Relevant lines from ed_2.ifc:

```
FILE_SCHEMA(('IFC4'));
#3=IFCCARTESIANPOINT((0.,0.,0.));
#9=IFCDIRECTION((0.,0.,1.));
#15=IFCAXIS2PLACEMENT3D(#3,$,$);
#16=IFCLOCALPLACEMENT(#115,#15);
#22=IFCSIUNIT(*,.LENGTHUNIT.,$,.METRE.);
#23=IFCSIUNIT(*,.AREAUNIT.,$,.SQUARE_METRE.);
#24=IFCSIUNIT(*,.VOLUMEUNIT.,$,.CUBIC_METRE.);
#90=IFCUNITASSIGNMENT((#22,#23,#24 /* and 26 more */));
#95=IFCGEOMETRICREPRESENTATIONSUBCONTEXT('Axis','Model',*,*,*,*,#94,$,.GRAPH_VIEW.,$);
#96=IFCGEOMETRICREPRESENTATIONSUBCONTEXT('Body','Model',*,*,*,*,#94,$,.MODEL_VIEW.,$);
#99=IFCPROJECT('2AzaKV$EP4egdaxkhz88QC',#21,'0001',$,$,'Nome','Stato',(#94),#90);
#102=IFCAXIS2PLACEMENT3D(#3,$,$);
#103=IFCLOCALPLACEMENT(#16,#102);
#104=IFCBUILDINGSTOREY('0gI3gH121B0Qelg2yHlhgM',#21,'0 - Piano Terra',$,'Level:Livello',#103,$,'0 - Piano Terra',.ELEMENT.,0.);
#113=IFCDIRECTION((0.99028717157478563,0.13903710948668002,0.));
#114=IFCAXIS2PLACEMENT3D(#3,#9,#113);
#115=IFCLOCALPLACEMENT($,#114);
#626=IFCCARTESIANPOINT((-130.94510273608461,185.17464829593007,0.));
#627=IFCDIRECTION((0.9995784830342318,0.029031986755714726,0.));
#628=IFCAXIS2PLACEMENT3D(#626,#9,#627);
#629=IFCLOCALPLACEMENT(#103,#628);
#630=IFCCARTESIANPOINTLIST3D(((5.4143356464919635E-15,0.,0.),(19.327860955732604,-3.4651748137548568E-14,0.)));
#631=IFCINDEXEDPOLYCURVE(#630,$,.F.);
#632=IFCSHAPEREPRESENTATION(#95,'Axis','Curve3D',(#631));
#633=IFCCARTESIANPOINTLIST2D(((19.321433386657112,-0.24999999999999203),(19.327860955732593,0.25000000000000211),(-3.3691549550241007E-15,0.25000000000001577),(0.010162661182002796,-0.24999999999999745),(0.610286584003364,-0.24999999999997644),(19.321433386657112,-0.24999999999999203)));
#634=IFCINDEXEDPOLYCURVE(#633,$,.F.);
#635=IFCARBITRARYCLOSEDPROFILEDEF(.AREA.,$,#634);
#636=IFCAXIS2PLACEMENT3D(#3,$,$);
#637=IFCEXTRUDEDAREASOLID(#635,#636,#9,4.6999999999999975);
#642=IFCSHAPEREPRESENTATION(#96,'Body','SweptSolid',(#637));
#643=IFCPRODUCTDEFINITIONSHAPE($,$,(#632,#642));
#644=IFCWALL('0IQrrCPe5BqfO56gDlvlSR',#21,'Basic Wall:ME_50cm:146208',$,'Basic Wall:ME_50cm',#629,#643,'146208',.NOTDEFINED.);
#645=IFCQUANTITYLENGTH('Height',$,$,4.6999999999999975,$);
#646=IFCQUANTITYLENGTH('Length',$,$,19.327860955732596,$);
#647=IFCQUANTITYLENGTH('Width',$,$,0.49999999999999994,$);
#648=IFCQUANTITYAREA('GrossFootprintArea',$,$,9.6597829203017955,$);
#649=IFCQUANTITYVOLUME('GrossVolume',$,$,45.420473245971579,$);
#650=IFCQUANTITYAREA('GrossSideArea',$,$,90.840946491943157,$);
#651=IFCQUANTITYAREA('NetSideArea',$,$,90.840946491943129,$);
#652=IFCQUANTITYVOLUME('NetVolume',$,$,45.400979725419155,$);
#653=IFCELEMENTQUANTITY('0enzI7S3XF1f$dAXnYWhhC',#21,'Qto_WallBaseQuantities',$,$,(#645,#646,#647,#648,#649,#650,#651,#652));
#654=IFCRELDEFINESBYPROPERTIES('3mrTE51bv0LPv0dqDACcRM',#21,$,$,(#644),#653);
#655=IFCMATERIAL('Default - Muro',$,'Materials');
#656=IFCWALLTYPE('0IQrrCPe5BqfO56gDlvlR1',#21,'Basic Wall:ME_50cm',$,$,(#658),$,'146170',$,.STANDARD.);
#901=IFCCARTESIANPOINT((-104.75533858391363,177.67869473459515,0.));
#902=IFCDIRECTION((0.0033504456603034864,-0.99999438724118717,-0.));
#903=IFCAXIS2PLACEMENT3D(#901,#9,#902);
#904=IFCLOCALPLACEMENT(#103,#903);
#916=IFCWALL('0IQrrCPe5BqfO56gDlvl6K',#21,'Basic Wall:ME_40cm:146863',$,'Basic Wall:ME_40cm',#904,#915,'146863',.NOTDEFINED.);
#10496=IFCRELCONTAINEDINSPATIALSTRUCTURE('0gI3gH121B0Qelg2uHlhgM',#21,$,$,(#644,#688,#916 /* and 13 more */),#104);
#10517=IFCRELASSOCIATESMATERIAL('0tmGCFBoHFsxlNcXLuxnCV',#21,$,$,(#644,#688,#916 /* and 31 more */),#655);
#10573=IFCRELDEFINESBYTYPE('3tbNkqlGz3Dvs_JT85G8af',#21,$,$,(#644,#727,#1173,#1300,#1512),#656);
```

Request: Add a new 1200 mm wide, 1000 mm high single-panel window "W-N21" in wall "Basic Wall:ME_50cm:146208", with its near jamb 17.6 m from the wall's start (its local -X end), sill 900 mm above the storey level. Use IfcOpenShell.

```python
import numpy as np
import ifcopenshell
import ifcopenshell.api.feature
import ifcopenshell.api.geometry
import ifcopenshell.api.pset
import ifcopenshell.api.root
import ifcopenshell.api.spatial
import ifcopenshell.geom
import ifcopenshell.util.element
import ifcopenshell.util.placement
import ifcopenshell.util.representation
import ifcopenshell.util.shape
import ifcopenshell.util.unit

model = ifcopenshell.open("ed_2.ifc")
unit_scale = ifcopenshell.util.unit.calculate_unit_scale(model)
area_scale = ifcopenshell.util.unit.calculate_unit_scale(model, "AREAUNIT")
volume_scale = ifcopenshell.util.unit.calculate_unit_scale(model, "VOLUMEUNIT")
settings = ifcopenshell.geom.settings()


def volume(element):
    """Net volume in cubic metres, openings subtracted."""
    shape = ifcopenshell.geom.create_shape(settings, element)
    return ifcopenshell.util.shape.get_volume(shape.geometry)


wall = model.by_guid("0IQrrCPe5BqfO56gDlvlSR")
storey = ifcopenshell.util.element.get_container(wall, ifc_class="IfcBuildingStorey")
context = ifcopenshell.util.representation.get_context(model, "Model", "Body", "MODEL_VIEW")
before = volume(wall)

width, height, from_end, sill = 1.2, 1, 17.6, 0.9  # metres

# The wall runs along its own X axis, and the end named is its -X end.
wall_shape = ifcopenshell.geom.create_shape(settings, wall)
x, y, z = ifcopenshell.util.shape.get_vertices(wall_shape.geometry).T
start = x.min() + from_end
face, thickness = float(y.min()), float(y.max() - y.min())
wall_matrix = ifcopenshell.util.placement.get_local_placement(wall.ObjectPlacement)
level = ifcopenshell.util.placement.get_local_placement(storey.ObjectPlacement)[2, 3]


def in_wall(x, y):
    """Placement at x, y metres in the wall's axes, at sill height."""
    matrix = wall_matrix.copy()
    matrix[:, 3] = wall_matrix @ np.array([x / unit_scale, y / unit_scale, 0.0, 1.0])
    matrix[2, 3] = level + sill / unit_scale
    return matrix


# Opening: a box that overshoots both wall faces by 50 mm.
opening = ifcopenshell.api.root.create_entity(model, ifc_class="IfcOpeningElement", predefined_type="OPENING")
box = ifcopenshell.api.geometry.add_wall_representation(
    model, context=context, length=width, height=height, thickness=thickness + 0.1
)
ifcopenshell.api.geometry.assign_representation(model, product=opening, representation=box)
ifcopenshell.api.geometry.edit_object_placement(model, product=opening, matrix=in_wall(start, face - 0.05), is_si=False)
ifcopenshell.api.feature.add_feature(model, feature=opening, element=wall)

window = ifcopenshell.api.root.create_entity(model, ifc_class="IfcWindow", name="W-N21", predefined_type="WINDOW")
window.OverallWidth, window.OverallHeight = width / unit_scale, height / unit_scale
window.PartitioningType = "SINGLE_PANEL"
body = ifcopenshell.api.geometry.add_window_representation(
    model,
    context=context,
    overall_width=window.OverallWidth,
    overall_height=window.OverallHeight,
    partition_type="SINGLE_PANEL",
)
ifcopenshell.api.geometry.assign_representation(model, product=window, representation=body)
ifcopenshell.api.spatial.assign_container(model, products=[window], relating_structure=storey)
ifcopenshell.api.feature.add_filling(model, opening=opening, element=window)

# Centre the window in the wall's thickness.
ifcopenshell.api.geometry.edit_object_placement(model, product=window, matrix=in_wall(start, face), is_si=False)
window_shape = ifcopenshell.geom.create_shape(settings, window)
depth = ifcopenshell.util.shape.get_vertices(window_shape.geometry)[:, 1]
offset = face + thickness / 2 - (depth.min() + depth.max()) / 2
ifcopenshell.api.geometry.edit_object_placement(model, product=window, matrix=in_wall(start, offset), is_si=False)

after = volume(wall)

# Update the wall's stored quantities.
qto = model.by_id(ifcopenshell.util.element.get_pset(wall, "Qto_WallBaseQuantities", should_inherit=False)["id"])
ifcopenshell.api.pset.edit_qto(model, qto=qto, properties={
    "NetSideArea": after / thickness / area_scale,
    "NetVolume": after / volume_scale,
})

print(f"wall volume {before:.3f} -> {after:.3f} m3")

model.write("ed_2_updated.ifc")
```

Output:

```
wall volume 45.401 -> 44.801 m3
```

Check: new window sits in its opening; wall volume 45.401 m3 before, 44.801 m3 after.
